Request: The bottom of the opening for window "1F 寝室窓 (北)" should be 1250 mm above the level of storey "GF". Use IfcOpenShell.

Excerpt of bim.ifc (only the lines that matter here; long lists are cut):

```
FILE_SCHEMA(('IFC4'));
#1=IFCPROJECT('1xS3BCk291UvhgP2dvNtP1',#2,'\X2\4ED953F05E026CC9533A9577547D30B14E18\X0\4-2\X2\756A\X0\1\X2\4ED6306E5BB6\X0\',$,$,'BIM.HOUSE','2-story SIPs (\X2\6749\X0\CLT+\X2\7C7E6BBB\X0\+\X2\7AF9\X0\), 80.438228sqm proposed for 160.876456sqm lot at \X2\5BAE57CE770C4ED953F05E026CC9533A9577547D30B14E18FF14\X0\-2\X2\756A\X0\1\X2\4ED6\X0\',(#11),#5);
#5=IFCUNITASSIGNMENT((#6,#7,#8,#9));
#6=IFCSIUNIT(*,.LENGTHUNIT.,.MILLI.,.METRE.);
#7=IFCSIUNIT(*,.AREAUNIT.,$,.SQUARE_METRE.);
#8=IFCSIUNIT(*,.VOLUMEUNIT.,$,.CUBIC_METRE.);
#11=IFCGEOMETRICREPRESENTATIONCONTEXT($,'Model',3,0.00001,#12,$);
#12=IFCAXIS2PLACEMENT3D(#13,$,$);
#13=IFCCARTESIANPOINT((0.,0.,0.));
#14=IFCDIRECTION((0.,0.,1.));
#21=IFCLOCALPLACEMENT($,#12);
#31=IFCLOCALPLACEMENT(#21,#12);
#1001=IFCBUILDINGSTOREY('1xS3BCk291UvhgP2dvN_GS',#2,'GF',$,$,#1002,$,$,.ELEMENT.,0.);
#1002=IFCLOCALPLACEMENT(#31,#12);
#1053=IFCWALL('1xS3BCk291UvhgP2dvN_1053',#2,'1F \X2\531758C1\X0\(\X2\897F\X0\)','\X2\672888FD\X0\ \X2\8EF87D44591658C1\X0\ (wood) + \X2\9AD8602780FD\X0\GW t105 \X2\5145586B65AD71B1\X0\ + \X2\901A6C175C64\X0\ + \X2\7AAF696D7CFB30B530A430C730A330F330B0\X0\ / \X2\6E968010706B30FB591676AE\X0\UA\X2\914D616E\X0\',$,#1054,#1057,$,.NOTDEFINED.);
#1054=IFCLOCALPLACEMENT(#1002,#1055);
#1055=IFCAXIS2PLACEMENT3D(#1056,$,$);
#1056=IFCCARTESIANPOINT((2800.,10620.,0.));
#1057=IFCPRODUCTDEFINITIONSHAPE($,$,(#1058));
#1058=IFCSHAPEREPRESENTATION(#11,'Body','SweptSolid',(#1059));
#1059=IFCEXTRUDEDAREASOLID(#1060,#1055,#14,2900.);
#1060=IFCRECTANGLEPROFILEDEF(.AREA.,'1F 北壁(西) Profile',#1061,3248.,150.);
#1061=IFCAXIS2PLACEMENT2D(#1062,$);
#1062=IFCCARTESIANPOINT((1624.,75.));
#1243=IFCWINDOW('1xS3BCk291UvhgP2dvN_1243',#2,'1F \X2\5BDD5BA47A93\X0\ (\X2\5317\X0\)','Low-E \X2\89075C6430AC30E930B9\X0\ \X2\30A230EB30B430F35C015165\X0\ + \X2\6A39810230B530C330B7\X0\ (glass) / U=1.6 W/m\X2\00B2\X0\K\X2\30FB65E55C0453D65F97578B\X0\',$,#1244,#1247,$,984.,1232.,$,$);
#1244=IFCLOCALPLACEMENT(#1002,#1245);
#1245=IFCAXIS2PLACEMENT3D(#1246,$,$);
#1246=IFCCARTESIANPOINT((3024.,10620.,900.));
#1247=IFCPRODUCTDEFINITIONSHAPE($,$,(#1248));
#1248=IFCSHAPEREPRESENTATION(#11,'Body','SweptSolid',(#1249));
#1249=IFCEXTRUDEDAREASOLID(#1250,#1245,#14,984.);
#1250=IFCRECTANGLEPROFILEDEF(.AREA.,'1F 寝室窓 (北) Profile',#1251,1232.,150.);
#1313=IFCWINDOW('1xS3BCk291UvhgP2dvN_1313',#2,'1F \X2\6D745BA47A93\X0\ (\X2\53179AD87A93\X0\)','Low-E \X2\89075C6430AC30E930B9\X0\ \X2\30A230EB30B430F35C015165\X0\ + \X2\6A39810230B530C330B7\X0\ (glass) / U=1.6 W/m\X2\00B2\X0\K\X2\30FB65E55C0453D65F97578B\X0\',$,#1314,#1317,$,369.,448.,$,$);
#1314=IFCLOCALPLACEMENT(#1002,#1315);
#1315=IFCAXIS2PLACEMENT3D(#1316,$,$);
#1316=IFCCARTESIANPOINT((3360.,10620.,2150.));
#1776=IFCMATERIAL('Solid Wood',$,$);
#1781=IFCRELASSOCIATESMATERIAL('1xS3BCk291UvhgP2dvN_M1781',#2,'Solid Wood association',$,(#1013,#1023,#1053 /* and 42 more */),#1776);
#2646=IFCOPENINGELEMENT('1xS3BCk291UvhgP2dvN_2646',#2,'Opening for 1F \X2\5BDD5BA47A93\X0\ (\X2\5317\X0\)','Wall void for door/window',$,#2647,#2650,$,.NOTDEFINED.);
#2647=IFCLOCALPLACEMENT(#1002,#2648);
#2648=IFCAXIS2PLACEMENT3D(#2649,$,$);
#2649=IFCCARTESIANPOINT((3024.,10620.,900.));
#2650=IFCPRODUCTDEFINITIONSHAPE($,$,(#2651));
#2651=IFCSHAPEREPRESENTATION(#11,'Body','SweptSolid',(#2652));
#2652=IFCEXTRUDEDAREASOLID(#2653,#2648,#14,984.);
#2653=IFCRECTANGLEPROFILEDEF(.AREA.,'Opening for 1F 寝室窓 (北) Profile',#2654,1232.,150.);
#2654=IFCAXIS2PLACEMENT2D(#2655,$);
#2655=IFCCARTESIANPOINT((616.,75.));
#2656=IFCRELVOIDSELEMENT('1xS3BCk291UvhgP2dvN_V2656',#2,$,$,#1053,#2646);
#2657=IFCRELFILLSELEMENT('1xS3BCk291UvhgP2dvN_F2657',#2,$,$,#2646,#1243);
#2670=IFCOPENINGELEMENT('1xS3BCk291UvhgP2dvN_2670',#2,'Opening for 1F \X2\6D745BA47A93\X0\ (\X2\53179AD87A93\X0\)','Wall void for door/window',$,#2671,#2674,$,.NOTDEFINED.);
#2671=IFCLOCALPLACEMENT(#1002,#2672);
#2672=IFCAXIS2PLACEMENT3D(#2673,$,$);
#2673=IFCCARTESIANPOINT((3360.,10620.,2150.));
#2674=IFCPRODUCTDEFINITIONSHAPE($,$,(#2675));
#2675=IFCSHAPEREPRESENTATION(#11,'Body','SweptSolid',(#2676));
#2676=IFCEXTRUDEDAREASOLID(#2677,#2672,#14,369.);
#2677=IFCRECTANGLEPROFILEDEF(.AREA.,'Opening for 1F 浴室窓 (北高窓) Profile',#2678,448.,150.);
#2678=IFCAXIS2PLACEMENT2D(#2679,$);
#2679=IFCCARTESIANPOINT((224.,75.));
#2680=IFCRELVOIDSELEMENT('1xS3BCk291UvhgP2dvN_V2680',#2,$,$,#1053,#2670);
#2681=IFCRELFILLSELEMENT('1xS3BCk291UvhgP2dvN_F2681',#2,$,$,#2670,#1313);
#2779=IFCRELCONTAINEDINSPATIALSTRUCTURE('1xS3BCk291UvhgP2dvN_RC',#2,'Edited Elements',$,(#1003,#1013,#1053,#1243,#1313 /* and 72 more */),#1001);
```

```python
import numpy as np
import ifcopenshell
import ifcopenshell.api.geometry
import ifcopenshell.geom
import ifcopenshell.util.element
import ifcopenshell.util.placement
import ifcopenshell.util.shape
import ifcopenshell.util.unit

model = ifcopenshell.open("bim.ifc")
unit_scale = ifcopenshell.util.unit.calculate_unit_scale(model)

window = model.by_guid("1xS3BCk291UvhgP2dvN_1243")
opening = window.FillsVoids[0].RelatingOpeningElement
storey = ifcopenshell.util.element.get_container(window, ifc_class="IfcBuildingStorey")
level = ifcopenshell.util.placement.get_local_placement(storey.ObjectPlacement)[2, 3]

# The opening's origin need not be at the sill, so measure its lowest point.
shape = ifcopenshell.geom.create_shape(ifcopenshell.geom.settings(), opening)
bottom = ifcopenshell.util.shape.get_shape_bottom_elevation(shape, shape.geometry) / unit_scale
dz = level + 1250.0 - bottom

shift = np.array([0.0, 0.0, dz])
# The window is not placed relative to its opening, so move both.
for product in (opening, window):
    matrix = ifcopenshell.util.placement.get_local_placement(product.ObjectPlacement)
    matrix[:3, 3] += shift
    ifcopenshell.api.geometry.edit_object_placement(model, product=product, matrix=matrix, is_si=False)

print(f"moved by {dz * unit_scale:+.3f} m")

model.write("bim-out.ifc")
```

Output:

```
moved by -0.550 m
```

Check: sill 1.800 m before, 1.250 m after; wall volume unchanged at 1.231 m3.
